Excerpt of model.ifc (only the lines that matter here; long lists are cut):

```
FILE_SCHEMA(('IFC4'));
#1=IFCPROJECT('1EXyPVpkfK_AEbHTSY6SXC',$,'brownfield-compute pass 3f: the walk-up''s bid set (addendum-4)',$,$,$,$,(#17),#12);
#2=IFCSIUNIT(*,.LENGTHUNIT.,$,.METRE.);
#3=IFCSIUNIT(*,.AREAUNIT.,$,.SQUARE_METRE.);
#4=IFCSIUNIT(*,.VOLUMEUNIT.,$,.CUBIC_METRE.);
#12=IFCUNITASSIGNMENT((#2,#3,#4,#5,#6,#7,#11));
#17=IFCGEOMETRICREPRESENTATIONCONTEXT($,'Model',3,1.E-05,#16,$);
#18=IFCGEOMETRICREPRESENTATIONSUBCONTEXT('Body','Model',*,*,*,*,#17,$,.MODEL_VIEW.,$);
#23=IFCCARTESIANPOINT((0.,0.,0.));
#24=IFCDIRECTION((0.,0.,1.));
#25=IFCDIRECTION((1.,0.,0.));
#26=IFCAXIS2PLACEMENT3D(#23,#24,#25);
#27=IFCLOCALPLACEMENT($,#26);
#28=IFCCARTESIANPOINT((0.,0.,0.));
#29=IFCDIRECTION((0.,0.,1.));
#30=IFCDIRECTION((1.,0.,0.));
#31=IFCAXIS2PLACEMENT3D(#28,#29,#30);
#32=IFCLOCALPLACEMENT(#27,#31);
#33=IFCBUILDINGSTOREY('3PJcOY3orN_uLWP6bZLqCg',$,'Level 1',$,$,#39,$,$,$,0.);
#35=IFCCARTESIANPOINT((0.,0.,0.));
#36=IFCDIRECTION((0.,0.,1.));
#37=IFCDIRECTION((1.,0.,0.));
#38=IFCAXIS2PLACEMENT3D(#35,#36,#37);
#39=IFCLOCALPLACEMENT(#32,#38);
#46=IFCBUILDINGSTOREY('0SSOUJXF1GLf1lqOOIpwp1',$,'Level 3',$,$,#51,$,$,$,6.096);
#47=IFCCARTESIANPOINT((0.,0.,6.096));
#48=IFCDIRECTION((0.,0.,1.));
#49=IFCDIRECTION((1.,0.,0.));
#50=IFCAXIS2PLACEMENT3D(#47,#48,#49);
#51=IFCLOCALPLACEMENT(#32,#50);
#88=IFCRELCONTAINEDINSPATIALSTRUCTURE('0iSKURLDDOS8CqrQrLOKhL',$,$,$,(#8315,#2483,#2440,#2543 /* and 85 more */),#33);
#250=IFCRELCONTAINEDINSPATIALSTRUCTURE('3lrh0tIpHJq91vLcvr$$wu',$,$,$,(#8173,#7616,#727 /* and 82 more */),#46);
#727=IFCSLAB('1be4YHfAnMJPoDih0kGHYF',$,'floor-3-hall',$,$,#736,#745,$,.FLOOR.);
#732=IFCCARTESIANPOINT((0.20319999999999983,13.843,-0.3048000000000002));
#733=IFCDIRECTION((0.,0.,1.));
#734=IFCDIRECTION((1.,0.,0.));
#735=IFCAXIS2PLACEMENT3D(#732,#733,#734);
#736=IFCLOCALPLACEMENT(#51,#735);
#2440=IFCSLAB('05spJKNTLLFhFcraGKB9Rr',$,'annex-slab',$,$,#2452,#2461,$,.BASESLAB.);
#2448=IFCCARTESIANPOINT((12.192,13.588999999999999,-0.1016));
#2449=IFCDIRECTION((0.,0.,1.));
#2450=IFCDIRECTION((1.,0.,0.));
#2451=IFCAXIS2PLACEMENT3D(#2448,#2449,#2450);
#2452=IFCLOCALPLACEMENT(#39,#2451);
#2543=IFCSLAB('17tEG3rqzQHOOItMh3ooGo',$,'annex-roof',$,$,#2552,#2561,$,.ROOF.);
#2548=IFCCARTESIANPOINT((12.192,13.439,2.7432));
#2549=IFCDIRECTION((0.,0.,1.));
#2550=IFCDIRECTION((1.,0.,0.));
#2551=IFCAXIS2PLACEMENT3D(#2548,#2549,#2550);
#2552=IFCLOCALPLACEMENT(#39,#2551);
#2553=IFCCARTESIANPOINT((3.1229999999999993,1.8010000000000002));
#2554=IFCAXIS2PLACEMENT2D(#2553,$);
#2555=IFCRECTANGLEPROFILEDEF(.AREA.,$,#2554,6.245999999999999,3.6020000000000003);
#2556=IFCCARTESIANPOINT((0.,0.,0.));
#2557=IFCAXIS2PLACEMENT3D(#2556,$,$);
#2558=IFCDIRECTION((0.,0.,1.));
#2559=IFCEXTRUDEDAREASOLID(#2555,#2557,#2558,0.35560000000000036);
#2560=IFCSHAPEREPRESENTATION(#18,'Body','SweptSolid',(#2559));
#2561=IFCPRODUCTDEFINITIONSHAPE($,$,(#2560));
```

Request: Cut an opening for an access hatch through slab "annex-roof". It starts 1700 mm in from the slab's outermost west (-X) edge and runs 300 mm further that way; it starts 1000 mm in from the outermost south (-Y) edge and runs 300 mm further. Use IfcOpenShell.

```python
import numpy as np
import ifcopenshell
import ifcopenshell.api.feature
import ifcopenshell.api.geometry
import ifcopenshell.api.root
import ifcopenshell.geom
import ifcopenshell.util.placement
import ifcopenshell.util.representation
import ifcopenshell.util.shape
import ifcopenshell.util.unit

model = ifcopenshell.open("model.ifc")
unit_scale = ifcopenshell.util.unit.calculate_unit_scale(model)
settings = ifcopenshell.geom.settings()


def volume(element):
    """Net volume in cubic metres, openings subtracted."""
    shape = ifcopenshell.geom.create_shape(settings, element)
    return ifcopenshell.util.shape.get_volume(shape.geometry)


slab = model.by_guid("17tEG3rqzQHOOItMh3ooGo")
before = volume(slab)

# Extent in the slab's own axes, in metres. The edges named are its -X and -Y sides.
slab_shape = ifcopenshell.geom.create_shape(settings, slab)
vertices = ifcopenshell.util.shape.get_vertices(slab_shape.geometry)
x_min, y_min, bottom = vertices.min(axis=0)
top = vertices[:, 2].max()

opening = ifcopenshell.api.root.create_entity(model, ifc_class="IfcOpeningElement", name="Access hatch opening", predefined_type="OPENING")
context = ifcopenshell.util.representation.get_context(model, "Model", "Body", "MODEL_VIEW")
width, depth = 0.3, 0.3
outline = [(0.0, 0.0), (width, 0.0), (width, depth), (0.0, depth), (0.0, 0.0)]
# Overshoot both faces by 50 mm so the cut is clean.
shape = ifcopenshell.api.geometry.add_slab_representation(
    model, context=context, depth=top - bottom + 0.1, polyline=outline
)
ifcopenshell.api.geometry.assign_representation(model, product=opening, representation=shape)

matrix = ifcopenshell.util.placement.get_local_placement(slab.ObjectPlacement)
matrix[:, 3] = matrix @ np.append(np.array([x_min + 1.7, y_min + 1, bottom - 0.05]) / unit_scale, 1.0)
ifcopenshell.api.geometry.edit_object_placement(model, product=opening, matrix=matrix, is_si=False)
ifcopenshell.api.feature.add_feature(model, feature=opening, element=slab)

after = volume(slab)

print(f"slab volume {before:.3f} -> {after:.3f} m3")

model.write("model-out.ifc")
```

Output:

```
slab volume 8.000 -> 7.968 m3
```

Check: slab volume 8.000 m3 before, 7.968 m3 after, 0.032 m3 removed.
